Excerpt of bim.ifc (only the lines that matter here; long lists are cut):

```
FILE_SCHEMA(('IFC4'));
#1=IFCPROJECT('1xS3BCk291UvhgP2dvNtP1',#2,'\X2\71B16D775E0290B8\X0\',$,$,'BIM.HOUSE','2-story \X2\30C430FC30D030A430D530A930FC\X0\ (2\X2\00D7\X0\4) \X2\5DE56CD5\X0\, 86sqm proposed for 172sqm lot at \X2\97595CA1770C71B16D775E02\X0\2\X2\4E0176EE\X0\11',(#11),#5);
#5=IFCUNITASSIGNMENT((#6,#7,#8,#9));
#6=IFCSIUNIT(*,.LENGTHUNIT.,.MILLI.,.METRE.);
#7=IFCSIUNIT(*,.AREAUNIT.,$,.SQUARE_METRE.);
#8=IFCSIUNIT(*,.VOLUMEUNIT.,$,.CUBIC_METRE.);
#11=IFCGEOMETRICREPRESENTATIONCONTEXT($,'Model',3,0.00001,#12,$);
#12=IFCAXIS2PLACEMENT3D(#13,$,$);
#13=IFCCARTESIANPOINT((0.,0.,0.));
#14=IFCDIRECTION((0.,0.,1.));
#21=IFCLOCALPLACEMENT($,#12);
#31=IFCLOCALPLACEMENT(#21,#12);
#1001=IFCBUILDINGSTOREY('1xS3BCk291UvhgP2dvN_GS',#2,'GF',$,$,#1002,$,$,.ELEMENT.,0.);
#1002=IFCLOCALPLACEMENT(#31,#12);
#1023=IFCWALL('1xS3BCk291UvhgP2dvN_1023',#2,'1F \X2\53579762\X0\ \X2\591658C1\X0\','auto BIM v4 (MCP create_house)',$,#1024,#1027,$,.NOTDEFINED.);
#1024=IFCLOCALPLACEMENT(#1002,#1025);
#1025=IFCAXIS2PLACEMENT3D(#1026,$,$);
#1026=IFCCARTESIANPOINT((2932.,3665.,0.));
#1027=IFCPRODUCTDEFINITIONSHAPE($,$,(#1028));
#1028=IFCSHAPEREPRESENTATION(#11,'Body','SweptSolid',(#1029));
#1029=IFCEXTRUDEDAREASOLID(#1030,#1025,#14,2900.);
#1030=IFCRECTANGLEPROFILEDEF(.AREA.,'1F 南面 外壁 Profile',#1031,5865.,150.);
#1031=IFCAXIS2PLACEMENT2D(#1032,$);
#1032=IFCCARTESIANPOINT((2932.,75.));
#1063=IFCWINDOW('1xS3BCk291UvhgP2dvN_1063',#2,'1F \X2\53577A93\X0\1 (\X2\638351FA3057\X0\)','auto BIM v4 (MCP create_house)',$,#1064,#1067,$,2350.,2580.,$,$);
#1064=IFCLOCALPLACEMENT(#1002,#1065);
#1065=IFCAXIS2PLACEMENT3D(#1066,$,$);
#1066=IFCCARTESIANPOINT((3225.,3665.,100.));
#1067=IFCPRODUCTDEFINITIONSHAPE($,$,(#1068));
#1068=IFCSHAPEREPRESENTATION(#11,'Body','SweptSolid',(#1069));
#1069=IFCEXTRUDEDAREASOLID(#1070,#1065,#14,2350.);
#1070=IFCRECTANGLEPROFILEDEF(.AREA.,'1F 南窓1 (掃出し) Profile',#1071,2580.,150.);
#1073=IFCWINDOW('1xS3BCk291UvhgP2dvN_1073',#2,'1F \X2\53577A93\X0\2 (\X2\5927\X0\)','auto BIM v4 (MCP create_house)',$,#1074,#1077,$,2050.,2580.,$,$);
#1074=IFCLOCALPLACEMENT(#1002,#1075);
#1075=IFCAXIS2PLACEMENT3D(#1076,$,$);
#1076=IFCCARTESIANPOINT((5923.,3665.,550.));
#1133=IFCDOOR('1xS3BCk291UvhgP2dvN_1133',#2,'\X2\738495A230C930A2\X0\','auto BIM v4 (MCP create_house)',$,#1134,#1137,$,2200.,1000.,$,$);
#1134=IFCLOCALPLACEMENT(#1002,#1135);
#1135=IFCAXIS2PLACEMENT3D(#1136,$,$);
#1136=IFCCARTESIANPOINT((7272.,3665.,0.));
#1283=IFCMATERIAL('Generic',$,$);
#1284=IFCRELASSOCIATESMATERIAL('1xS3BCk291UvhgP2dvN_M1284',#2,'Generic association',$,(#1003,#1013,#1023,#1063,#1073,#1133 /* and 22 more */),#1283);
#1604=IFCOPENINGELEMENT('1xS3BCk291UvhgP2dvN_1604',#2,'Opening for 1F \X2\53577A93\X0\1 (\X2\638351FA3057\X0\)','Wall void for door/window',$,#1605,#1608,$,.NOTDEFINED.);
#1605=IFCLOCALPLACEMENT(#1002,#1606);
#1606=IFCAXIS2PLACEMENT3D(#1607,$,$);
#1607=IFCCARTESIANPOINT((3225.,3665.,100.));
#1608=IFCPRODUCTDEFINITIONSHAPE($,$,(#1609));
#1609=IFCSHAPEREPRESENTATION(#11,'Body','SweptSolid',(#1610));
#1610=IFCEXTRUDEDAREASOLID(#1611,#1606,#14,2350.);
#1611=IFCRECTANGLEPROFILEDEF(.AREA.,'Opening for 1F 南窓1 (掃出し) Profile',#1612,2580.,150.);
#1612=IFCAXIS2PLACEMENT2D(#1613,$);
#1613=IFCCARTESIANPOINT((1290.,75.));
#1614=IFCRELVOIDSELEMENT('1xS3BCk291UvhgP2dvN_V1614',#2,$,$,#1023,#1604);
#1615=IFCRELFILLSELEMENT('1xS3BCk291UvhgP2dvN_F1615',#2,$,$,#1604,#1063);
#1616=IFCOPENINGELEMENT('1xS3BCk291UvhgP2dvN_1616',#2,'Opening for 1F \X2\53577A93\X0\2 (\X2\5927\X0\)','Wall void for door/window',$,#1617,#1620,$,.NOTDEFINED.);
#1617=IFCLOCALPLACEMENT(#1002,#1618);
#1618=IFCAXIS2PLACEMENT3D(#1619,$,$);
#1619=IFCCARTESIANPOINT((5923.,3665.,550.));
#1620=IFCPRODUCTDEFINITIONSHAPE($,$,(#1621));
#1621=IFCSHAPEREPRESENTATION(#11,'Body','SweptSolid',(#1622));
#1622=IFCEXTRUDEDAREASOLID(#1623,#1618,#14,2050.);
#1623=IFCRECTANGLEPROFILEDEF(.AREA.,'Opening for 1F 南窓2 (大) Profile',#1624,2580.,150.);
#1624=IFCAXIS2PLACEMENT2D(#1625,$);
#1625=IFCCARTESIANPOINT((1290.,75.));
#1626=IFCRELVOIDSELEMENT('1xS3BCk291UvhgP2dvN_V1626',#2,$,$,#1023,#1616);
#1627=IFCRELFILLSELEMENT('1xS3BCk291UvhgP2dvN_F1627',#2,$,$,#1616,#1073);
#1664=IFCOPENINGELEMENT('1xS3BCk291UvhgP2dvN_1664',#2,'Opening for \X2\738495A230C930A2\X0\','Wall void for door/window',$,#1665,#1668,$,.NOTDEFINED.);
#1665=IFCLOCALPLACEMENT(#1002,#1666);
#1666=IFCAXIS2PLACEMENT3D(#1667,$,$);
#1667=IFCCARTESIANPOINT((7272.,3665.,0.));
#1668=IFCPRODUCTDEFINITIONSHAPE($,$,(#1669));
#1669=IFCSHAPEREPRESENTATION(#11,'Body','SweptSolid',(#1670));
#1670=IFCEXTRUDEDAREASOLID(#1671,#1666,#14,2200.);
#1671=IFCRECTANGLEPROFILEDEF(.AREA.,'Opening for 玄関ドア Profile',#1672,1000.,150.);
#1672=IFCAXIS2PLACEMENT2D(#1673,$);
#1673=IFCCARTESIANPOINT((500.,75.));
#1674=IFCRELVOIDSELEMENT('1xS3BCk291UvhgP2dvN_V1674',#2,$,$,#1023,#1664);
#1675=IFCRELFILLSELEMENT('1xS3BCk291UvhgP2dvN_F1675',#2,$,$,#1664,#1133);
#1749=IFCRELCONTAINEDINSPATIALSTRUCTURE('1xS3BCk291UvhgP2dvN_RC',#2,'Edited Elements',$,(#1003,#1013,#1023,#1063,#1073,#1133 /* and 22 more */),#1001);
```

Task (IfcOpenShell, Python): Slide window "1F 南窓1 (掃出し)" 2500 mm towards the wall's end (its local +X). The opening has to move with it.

```python
import ifcopenshell
import ifcopenshell.api.geometry
import ifcopenshell.util.placement
import ifcopenshell.util.unit

model = ifcopenshell.open("bim.ifc")
unit_scale = ifcopenshell.util.unit.calculate_unit_scale(model)

window = model.by_guid("1xS3BCk291UvhgP2dvN_1063")
opening = window.FillsVoids[0].RelatingOpeningElement
wall = opening.VoidsElements[0].RelatingBuildingElement

wall_matrix = ifcopenshell.util.placement.get_local_placement(wall.ObjectPlacement)
shift = wall_matrix[:3, 0] * 2.5 / unit_scale
before = ifcopenshell.util.placement.get_local_placement(window.ObjectPlacement)[:3, 3].copy()

# The window is not placed relative to its opening, so move both.
for product in (opening, window):
    matrix = ifcopenshell.util.placement.get_local_placement(product.ObjectPlacement)
    matrix[:3, 3] += shift
    ifcopenshell.api.geometry.edit_object_placement(model, product=product, matrix=matrix, is_si=False)

after = ifcopenshell.util.placement.get_local_placement(window.ObjectPlacement)[:3, 3]
print("window moved by", (after - before).round(3) + 0.0)

model.write("bim_updated.ifc")
```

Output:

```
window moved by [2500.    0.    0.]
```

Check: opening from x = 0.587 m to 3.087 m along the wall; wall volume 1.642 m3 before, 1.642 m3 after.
